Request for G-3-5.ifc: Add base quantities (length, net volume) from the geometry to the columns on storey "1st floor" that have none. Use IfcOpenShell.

First a look at what the model holds.

```python
import ifcopenshell
import ifcopenshell.util.element
import ifcopenshell.util.unit

model = ifcopenshell.open("G-3-5.ifc")
print(model.schema)
for unit_type in ("LENGTHUNIT", "AREAUNIT", "VOLUMEUNIT"):
    print(unit_type, ifcopenshell.util.unit.calculate_unit_scale(model, unit_type))
storey = next(s for s in model.by_type("IfcBuildingStorey") if s.Name == "1st floor")
columns = [e for e in ifcopenshell.util.element.get_decomposition(storey) if e.is_a("IfcColumn")]
for e in sorted(columns, key=lambda e: e.id()):
    print(e.id(), e.is_a(), e.Name, list(ifcopenshell.util.element.get_psets(e, qtos_only=True)), sep=" | ")
```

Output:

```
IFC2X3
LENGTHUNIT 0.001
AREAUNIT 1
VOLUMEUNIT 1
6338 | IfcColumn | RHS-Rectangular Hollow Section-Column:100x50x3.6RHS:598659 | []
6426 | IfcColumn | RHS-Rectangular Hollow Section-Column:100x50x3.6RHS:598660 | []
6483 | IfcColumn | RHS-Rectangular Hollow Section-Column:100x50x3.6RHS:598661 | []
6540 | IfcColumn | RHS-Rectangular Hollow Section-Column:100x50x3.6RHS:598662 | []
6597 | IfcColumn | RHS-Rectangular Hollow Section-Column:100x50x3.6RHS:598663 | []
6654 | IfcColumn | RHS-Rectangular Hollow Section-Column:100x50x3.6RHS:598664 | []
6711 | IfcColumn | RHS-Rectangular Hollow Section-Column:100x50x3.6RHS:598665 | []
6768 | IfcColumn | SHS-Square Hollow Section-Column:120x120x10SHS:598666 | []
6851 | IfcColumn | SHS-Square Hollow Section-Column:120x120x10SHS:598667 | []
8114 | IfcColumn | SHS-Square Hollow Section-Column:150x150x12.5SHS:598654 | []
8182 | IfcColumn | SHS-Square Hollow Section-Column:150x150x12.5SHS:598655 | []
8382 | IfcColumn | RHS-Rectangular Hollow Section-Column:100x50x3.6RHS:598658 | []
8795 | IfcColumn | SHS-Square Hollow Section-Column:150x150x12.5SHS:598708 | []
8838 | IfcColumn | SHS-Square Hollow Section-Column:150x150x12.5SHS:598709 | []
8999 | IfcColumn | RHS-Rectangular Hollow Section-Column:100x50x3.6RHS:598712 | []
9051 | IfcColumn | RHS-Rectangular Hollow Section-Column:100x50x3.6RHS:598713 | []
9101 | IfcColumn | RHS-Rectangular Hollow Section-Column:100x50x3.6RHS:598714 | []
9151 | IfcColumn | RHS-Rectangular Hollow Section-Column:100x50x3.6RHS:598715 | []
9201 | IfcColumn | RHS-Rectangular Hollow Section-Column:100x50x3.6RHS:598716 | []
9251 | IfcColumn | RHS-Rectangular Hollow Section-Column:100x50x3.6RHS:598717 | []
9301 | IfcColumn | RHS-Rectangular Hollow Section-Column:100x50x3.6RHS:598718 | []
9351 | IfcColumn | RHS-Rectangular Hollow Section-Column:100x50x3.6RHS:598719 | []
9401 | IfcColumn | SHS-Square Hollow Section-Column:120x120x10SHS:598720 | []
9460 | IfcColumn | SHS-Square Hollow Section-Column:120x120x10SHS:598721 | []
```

```python
import ifcopenshell
import ifcopenshell.api.pset
import ifcopenshell.geom
import ifcopenshell.util.element
import ifcopenshell.util.shape
import ifcopenshell.util.unit

model = ifcopenshell.open("G-3-5.ifc")
unit_scale = ifcopenshell.util.unit.calculate_unit_scale(model)
volume_scale = ifcopenshell.util.unit.calculate_unit_scale(model, "VOLUMEUNIT")
settings = ifcopenshell.geom.settings()

storey = next(s for s in model.by_type("IfcBuildingStorey") if s.Name == "1st floor")
columns = [e for e in ifcopenshell.util.element.get_decomposition(storey) if e.is_a("IfcColumn")]

for e in sorted(columns, key=lambda e: e.id()):
    if ifcopenshell.util.element.get_psets(e, qtos_only=True, should_inherit=False):
        continue
    # Geometry comes back in metres, in the element's own axes.
    shape = ifcopenshell.geom.create_shape(settings, e)
    values = {
        "Length": ifcopenshell.util.shape.get_z(shape.geometry) / unit_scale,
        "NetVolume": ifcopenshell.util.shape.get_volume(shape.geometry) / volume_scale,
    }
    qto = ifcopenshell.api.pset.add_qto(model, product=e, name="BaseQuantities")
    ifcopenshell.api.pset.edit_qto(model, qto=qto, properties=values)
    print(e.id(), {k: round(v, 3) for k, v in values.items()})

model.write("G-3-5_edited.ifc")
```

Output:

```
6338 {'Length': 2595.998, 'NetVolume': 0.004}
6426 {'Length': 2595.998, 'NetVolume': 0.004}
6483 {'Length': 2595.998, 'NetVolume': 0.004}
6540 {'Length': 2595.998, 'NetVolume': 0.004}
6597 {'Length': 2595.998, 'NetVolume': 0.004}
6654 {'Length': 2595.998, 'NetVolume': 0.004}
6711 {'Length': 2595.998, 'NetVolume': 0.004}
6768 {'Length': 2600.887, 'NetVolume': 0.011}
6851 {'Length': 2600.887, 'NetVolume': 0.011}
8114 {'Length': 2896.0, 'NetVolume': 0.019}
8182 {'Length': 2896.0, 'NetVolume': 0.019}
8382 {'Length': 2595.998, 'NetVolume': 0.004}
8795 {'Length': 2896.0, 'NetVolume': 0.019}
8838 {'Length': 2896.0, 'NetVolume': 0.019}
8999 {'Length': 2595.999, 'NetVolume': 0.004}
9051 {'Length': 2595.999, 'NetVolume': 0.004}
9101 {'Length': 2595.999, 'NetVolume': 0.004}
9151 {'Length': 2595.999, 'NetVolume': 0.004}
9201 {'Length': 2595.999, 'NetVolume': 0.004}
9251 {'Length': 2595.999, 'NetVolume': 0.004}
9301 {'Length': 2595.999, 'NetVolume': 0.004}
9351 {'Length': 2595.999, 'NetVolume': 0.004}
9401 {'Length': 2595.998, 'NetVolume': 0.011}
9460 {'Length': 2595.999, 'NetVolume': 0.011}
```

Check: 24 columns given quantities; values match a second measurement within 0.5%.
